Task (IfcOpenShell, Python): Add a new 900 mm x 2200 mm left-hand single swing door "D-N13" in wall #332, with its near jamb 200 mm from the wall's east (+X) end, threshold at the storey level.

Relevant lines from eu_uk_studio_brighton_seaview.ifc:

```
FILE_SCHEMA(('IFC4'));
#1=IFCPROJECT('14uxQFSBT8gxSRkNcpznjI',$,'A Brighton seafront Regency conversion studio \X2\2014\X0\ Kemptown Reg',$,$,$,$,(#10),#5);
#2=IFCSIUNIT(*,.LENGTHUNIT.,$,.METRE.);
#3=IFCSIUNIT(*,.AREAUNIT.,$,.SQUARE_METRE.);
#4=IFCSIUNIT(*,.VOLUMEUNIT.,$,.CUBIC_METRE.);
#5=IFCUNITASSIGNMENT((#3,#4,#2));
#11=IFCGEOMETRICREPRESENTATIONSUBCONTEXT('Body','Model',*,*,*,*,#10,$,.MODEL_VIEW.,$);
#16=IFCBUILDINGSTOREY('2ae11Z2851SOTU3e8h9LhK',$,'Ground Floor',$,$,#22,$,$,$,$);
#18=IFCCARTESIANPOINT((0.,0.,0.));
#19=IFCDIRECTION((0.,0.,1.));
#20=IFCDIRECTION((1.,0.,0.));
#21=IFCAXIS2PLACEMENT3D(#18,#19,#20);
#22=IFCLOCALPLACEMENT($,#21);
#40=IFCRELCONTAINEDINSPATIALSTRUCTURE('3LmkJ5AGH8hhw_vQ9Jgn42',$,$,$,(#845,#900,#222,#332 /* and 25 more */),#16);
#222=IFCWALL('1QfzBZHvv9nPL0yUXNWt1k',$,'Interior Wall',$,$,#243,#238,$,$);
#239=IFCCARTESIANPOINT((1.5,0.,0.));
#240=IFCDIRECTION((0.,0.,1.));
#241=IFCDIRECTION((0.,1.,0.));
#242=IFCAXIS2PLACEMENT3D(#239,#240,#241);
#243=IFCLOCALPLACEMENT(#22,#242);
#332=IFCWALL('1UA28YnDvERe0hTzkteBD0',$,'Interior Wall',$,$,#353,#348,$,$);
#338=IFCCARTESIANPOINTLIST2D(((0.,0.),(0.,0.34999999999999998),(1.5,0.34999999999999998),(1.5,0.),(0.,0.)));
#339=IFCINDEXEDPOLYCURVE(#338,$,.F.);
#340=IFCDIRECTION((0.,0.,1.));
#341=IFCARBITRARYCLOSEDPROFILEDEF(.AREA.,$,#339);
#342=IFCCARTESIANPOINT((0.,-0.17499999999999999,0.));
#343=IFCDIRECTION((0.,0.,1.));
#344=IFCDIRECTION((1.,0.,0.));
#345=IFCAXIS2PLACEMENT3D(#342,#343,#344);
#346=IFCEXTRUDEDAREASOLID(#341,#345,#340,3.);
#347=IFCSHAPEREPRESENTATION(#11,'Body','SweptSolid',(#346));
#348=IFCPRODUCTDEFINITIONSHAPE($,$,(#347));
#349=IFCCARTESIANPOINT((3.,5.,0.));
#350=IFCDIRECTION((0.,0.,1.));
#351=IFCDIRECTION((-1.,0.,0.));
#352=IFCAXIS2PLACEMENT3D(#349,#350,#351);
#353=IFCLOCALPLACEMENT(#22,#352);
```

```python
import numpy as np
import ifcopenshell
import ifcopenshell.api.feature
import ifcopenshell.api.geometry
import ifcopenshell.api.root
import ifcopenshell.api.spatial
import ifcopenshell.geom
import ifcopenshell.util.element
import ifcopenshell.util.placement
import ifcopenshell.util.representation
import ifcopenshell.util.shape
import ifcopenshell.util.unit

model = ifcopenshell.open("eu_uk_studio_brighton_seaview.ifc")
unit_scale = ifcopenshell.util.unit.calculate_unit_scale(model)
settings = ifcopenshell.geom.settings()


def volume(element):
    """Net volume in cubic metres, openings subtracted."""
    shape = ifcopenshell.geom.create_shape(settings, element)
    return ifcopenshell.util.shape.get_volume(shape.geometry)


wall = model.by_guid("1UA28YnDvERe0hTzkteBD0")
storey = ifcopenshell.util.element.get_container(wall, ifc_class="IfcBuildingStorey")
context = ifcopenshell.util.representation.get_context(model, "Model", "Body", "MODEL_VIEW")
before = volume(wall)

width, height, from_end, sill = 0.9, 2.2, 0.2, 0.0  # metres

# The wall runs along its own X axis, and the end named is its -X end.
wall_shape = ifcopenshell.geom.create_shape(settings, wall)
x, y, z = ifcopenshell.util.shape.get_vertices(wall_shape.geometry).T
start = x.min() + from_end
face, thickness = float(y.min()), float(y.max() - y.min())
wall_matrix = ifcopenshell.util.placement.get_local_placement(wall.ObjectPlacement)
level = ifcopenshell.util.placement.get_local_placement(storey.ObjectPlacement)[2, 3]


def in_wall(x, y):
    """Placement at x, y metres in the wall's axes, at sill height."""
    matrix = wall_matrix.copy()
    matrix[:, 3] = wall_matrix @ np.array([x / unit_scale, y / unit_scale, 0.0, 1.0])
    matrix[2, 3] = level + sill / unit_scale
    return matrix


# Opening: a box that overshoots both wall faces by 50 mm.
opening = ifcopenshell.api.root.create_entity(model, ifc_class="IfcOpeningElement", predefined_type="OPENING")
box = ifcopenshell.api.geometry.add_wall_representation(
    model, context=context, length=width, height=height, thickness=thickness + 0.1
)
ifcopenshell.api.geometry.assign_representation(model, product=opening, representation=box)
ifcopenshell.api.geometry.edit_object_placement(model, product=opening, matrix=in_wall(start, face - 0.05), is_si=False)
ifcopenshell.api.feature.add_feature(model, feature=opening, element=wall)

door = ifcopenshell.api.root.create_entity(model, ifc_class="IfcDoor", name="D-N13", predefined_type="DOOR")
door.OverallWidth, door.OverallHeight = width / unit_scale, height / unit_scale
door.OperationType = "SINGLE_SWING_LEFT"
body = ifcopenshell.api.geometry.add_door_representation(
    model,
    context=context,
    overall_width=door.OverallWidth,
    overall_height=door.OverallHeight,
    operation_type="SINGLE_SWING_LEFT",
    lining_properties={"LiningDepth": thickness / unit_scale, "ThresholdDepth": thickness / unit_scale},
)
ifcopenshell.api.geometry.assign_representation(model, product=door, representation=body)
ifcopenshell.api.spatial.assign_container(model, products=[door], relating_structure=storey)
ifcopenshell.api.feature.add_filling(model, opening=opening, element=door)

# The lining spans the wall, so the door starts at the wall face.
ifcopenshell.api.geometry.edit_object_placement(model, product=door, matrix=in_wall(start, face), is_si=False)

after = volume(wall)

print(f"wall volume {before:.3f} -> {after:.3f} m3")

model.write("eu_uk_studio_brighton_seaview_v2.ifc")
```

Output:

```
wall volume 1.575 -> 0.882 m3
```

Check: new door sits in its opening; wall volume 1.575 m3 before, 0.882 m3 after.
